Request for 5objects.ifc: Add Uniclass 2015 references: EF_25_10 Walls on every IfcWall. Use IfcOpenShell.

First a look at what the model holds.

```python
import ifcopenshell

model = ifcopenshell.open("5objects.ifc")
print(model.schema)
print("classifications:", [c.Name for c in model.by_type("IfcClassification")])
for ifc_class in ("IfcDoor", "IfcRoof", "IfcStair", "IfcWall", "IfcWindow"):
    print(ifc_class, len(model.by_type(ifc_class)))
```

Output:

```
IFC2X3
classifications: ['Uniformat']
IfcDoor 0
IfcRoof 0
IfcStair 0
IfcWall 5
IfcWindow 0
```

```python
import ifcopenshell
import ifcopenshell.api.classification

model = ifcopenshell.open("5objects.ifc")

# IFC2X3 requires Source and Edition and has no link from the project to the system.
system = model.create_entity("IfcClassification", Source="NBS", Edition="2015", Name="Uniclass 2015")

codes = {
    "IfcWall": ("EF_25_10", "Walls"),
}
for ifc_class, (code, name) in codes.items():
    products = model.by_type(ifc_class)
    ifcopenshell.api.classification.add_reference(
        model, products=products, classification=system, identification=code, name=name
    )
    print(code, len(products))

model.write("5objects_edited.ifc")
```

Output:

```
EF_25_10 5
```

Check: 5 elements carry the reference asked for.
